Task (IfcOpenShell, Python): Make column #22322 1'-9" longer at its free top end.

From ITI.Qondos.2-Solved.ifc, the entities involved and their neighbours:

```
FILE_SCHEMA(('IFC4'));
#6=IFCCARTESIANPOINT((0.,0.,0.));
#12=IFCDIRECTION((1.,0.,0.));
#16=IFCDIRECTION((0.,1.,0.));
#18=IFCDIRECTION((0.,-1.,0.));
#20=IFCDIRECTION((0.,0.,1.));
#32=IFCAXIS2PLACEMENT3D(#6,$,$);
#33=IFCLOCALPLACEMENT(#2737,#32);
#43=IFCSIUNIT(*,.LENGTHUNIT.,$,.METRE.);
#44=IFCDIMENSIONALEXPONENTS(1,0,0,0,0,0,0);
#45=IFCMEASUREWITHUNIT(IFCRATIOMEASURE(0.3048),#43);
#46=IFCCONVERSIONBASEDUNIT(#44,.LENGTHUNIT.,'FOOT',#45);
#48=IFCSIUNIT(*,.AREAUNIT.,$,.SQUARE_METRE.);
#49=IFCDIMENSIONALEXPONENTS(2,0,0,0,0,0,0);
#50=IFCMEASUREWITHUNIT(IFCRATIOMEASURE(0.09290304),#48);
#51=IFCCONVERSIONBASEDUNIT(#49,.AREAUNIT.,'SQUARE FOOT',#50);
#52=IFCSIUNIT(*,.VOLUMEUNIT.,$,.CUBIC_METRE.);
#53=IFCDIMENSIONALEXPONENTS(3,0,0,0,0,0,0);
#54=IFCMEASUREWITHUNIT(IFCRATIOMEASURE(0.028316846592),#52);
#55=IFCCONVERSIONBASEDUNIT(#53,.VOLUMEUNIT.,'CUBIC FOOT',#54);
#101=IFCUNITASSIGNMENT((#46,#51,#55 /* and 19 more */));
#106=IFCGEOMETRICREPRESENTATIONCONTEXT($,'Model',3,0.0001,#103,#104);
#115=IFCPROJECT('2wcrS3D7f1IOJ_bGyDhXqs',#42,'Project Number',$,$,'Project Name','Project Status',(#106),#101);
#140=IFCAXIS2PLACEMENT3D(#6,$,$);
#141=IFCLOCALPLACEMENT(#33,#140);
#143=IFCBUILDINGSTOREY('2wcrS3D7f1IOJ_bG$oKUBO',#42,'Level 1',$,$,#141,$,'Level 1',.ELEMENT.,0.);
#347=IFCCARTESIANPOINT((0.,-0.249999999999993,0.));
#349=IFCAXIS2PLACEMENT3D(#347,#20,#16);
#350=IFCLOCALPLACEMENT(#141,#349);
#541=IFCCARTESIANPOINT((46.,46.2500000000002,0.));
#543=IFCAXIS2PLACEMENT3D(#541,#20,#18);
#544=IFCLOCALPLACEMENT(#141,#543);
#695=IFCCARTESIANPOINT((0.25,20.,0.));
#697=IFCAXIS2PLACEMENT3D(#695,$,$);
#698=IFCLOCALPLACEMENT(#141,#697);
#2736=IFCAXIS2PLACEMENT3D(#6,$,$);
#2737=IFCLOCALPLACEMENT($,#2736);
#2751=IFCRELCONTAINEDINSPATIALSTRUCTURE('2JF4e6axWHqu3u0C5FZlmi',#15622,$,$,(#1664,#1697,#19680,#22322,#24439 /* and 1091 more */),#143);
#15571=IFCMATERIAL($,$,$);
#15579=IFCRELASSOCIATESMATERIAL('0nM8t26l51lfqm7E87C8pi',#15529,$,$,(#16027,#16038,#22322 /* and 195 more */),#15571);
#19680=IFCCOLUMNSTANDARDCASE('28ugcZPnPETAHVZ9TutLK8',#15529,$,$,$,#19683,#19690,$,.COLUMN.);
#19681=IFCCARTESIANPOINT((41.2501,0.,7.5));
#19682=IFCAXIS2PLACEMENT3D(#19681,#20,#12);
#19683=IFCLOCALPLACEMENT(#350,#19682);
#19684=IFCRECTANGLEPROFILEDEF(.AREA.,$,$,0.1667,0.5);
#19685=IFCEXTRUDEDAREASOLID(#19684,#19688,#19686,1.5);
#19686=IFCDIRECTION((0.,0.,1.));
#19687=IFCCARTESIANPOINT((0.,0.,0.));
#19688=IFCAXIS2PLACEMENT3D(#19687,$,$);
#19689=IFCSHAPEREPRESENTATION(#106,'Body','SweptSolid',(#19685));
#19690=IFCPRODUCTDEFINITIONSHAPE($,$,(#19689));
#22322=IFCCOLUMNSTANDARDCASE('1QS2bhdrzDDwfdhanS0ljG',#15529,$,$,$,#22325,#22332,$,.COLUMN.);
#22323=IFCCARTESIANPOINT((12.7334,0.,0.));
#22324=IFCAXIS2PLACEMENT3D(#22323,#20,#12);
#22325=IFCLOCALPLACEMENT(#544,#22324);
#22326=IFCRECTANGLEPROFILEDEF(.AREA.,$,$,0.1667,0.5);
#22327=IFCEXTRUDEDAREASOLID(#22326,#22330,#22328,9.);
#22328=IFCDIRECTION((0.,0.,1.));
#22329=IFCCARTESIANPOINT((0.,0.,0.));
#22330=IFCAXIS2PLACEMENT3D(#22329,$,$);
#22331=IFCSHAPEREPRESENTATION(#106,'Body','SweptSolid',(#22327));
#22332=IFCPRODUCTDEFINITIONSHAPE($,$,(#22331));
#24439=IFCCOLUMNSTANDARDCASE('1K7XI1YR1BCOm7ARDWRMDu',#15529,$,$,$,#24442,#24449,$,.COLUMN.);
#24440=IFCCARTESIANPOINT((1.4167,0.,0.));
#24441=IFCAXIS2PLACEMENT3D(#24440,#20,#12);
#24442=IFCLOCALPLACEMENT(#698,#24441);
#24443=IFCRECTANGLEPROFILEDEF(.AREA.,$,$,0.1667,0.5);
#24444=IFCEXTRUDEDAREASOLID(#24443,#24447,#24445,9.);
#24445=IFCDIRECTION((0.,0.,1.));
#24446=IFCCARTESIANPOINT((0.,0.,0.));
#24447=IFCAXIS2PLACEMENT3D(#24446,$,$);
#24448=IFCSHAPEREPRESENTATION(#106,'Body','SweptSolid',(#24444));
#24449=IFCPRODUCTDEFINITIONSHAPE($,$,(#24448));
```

```python
import ifcopenshell
import ifcopenshell.util.unit

model = ifcopenshell.open("ITI.Qondos.2-Solved.ifc")
unit_scale = ifcopenshell.util.unit.calculate_unit_scale(model)

member = model.by_guid("1QS2bhdrzDDwfdhanS0ljG")
change = 21 * 0.0254 / unit_scale

# The extrusion runs towards the end named, so only its depth changes.
body = next(r for r in member.Representation.Representations if r.RepresentationIdentifier == "Body")
solid = body.Items[0]
old_length = solid.Depth
solid.Depth += change

print(f"length {old_length:g} -> {solid.Depth:g}")

model.write("ITI.Qondos.2-Solved_rev.ifc")
```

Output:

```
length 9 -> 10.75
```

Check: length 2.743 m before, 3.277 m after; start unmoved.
